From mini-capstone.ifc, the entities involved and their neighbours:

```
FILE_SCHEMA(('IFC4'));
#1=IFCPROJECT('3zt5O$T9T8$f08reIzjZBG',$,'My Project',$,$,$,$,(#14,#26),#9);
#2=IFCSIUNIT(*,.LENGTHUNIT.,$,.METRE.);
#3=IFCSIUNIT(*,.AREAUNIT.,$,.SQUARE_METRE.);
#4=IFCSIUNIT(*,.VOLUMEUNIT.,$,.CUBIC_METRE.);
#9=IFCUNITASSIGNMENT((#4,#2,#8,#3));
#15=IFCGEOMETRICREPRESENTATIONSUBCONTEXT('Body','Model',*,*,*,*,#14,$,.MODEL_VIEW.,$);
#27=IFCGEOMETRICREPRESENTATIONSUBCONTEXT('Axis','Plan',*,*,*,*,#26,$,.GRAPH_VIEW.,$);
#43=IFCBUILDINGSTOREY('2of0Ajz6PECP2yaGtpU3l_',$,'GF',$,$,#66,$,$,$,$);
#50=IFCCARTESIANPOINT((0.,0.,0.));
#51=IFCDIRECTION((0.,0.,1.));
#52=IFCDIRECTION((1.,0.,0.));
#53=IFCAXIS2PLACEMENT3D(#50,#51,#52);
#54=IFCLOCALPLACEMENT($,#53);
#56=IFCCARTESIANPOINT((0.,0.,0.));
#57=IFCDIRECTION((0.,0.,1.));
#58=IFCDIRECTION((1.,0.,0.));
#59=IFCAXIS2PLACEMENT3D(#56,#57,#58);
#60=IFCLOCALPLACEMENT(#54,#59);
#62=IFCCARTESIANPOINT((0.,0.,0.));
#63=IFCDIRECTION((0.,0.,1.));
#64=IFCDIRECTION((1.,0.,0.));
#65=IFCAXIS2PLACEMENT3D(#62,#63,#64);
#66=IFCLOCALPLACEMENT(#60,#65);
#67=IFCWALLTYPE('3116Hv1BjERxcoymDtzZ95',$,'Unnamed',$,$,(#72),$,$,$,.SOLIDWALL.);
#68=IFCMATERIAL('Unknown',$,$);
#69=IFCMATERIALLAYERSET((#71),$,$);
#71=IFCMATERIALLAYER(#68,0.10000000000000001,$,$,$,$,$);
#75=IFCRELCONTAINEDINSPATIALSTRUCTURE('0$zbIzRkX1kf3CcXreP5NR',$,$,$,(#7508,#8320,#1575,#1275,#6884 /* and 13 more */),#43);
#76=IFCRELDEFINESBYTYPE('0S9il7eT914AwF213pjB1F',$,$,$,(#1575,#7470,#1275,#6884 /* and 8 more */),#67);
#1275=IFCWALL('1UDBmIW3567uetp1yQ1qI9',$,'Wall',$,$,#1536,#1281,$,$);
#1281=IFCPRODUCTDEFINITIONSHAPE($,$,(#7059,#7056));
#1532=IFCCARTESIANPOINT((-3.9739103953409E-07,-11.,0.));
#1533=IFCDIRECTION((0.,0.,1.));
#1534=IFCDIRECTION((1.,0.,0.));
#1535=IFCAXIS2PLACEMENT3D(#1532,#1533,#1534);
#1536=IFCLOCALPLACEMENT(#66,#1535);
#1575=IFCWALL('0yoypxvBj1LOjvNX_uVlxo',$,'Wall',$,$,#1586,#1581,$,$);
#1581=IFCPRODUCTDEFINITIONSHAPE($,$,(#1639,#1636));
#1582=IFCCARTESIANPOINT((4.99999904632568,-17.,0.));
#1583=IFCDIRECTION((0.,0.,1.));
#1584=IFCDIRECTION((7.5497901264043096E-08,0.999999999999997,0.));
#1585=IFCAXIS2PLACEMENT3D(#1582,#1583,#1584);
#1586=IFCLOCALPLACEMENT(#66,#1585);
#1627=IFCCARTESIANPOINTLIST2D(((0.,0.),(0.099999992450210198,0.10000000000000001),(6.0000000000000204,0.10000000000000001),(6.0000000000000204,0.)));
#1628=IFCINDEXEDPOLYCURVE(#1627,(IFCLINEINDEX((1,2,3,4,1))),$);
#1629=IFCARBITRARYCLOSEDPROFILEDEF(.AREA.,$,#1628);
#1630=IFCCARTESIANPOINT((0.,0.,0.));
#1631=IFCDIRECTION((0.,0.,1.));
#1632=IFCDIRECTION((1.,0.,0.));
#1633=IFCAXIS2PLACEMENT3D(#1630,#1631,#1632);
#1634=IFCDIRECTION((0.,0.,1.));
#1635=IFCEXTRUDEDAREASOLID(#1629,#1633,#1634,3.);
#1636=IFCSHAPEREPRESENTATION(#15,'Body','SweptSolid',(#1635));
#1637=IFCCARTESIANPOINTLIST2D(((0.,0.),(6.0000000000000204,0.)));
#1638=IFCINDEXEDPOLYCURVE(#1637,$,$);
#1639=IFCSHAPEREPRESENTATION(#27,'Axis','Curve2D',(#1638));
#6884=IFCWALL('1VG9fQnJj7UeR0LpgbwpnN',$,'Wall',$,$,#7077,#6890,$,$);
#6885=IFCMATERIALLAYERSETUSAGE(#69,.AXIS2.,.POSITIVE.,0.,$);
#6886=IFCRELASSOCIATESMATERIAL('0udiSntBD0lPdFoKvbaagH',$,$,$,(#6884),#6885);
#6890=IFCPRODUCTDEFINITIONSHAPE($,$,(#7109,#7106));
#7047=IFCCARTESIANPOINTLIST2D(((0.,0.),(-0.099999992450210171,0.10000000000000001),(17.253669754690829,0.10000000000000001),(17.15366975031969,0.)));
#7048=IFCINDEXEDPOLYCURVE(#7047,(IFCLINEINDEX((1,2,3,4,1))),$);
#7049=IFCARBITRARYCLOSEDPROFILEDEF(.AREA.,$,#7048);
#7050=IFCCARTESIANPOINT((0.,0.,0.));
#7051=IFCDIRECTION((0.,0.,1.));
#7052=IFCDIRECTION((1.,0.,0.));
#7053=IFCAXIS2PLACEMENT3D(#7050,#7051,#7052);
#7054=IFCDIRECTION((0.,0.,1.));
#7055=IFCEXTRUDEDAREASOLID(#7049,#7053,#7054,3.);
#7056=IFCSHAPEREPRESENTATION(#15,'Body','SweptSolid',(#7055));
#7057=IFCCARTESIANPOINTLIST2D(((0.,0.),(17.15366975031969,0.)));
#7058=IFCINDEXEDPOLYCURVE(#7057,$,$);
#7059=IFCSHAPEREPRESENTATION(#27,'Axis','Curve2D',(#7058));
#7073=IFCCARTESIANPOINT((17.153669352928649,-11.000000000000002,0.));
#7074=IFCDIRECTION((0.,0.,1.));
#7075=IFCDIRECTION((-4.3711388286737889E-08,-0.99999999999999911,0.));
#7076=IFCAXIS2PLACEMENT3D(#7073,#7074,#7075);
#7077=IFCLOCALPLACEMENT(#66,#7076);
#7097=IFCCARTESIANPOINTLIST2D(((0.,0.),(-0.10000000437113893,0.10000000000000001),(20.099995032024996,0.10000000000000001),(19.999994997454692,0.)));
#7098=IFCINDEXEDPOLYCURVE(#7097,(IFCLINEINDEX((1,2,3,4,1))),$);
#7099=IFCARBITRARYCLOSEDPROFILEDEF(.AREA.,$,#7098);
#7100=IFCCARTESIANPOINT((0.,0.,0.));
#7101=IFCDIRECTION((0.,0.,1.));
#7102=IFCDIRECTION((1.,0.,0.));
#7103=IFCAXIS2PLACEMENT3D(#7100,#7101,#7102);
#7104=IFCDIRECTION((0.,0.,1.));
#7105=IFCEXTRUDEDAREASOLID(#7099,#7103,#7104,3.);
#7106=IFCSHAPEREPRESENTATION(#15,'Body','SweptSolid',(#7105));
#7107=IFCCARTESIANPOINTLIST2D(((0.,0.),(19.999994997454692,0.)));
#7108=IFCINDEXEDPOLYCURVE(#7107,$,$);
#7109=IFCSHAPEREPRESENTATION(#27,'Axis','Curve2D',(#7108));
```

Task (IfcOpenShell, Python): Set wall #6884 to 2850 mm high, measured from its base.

```python
import ifcopenshell
import ifcopenshell.geom
import ifcopenshell.util.representation
import ifcopenshell.util.shape

model = ifcopenshell.open("mini-capstone.ifc")
settings = ifcopenshell.geom.settings()


def volume(element):
    """Net volume in cubic metres, openings subtracted."""
    shape = ifcopenshell.geom.create_shape(settings, element)
    return ifcopenshell.util.shape.get_volume(shape.geometry)


wall = model.by_id(6884)
before = volume(wall)

body = ifcopenshell.util.representation.get_representation(wall, "Model", "Body")
solid = body.Items[0]
old_height = solid.Depth
solid.Depth = 2.85
after = volume(wall)

print(f"height {old_height:g} -> {solid.Depth:g}, volume {before:.3f} -> {after:.3f} m3")

model.write("mini-capstone_updated.ifc")
```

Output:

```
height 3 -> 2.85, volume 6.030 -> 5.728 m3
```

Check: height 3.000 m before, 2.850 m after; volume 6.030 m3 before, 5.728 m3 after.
